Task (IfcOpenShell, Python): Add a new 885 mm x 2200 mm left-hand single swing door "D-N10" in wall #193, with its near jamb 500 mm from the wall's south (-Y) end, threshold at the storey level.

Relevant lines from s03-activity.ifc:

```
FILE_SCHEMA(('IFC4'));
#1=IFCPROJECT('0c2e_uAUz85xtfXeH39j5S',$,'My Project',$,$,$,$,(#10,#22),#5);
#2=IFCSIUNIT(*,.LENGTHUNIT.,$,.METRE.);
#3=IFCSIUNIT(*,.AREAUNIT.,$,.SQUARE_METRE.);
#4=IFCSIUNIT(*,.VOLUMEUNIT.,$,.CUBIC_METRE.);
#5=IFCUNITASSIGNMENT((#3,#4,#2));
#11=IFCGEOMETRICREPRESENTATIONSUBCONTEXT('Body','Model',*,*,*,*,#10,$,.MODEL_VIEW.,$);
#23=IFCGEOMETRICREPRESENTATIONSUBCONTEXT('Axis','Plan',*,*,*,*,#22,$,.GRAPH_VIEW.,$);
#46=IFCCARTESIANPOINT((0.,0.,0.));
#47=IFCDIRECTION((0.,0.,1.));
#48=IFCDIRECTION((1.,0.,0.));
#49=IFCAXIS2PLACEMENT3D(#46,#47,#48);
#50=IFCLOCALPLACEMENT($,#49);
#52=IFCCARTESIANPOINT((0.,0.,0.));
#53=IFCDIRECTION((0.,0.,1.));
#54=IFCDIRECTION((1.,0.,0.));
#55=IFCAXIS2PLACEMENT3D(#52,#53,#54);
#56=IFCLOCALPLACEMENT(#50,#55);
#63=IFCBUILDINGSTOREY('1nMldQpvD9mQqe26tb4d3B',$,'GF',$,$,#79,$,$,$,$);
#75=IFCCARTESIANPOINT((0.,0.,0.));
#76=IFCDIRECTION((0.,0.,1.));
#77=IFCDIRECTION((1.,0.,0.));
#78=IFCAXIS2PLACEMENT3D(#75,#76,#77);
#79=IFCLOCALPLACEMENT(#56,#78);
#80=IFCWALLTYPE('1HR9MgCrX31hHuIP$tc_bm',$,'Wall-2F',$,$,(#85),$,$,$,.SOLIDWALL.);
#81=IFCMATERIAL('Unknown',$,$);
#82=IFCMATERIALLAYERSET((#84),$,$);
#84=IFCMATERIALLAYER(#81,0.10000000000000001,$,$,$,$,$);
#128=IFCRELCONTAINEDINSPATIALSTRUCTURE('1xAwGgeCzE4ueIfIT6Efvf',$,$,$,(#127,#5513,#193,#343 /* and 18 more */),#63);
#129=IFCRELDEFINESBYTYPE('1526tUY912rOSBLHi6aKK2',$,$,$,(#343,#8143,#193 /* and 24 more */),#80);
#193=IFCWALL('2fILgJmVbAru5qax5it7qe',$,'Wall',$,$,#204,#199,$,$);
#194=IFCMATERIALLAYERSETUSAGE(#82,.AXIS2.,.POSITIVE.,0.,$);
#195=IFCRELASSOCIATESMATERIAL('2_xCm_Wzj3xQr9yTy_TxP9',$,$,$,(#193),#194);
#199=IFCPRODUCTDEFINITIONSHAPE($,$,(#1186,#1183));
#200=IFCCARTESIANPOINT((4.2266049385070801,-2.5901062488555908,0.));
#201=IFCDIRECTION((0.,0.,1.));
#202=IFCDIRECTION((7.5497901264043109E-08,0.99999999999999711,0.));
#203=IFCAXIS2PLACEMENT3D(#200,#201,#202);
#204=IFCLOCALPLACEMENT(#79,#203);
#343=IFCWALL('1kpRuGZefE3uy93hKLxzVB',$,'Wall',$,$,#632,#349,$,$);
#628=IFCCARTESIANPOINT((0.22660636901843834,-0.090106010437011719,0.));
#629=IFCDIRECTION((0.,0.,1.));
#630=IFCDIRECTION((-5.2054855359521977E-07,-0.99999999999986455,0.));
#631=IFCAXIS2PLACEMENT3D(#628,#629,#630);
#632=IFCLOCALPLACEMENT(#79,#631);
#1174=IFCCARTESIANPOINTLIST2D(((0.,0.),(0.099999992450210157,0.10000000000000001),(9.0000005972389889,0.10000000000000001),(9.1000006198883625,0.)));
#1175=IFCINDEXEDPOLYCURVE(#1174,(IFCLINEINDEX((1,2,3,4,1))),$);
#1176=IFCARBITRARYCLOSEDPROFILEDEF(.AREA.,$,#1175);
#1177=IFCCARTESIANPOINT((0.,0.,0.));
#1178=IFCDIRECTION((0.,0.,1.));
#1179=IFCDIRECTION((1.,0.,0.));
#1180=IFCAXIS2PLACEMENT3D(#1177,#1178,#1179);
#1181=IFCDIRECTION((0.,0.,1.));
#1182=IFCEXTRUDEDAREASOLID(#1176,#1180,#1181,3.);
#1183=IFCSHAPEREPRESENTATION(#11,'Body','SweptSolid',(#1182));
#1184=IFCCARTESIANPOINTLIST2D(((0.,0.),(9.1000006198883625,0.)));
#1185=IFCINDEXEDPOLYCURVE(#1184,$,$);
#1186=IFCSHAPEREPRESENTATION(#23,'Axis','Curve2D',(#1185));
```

```python
import numpy as np
import ifcopenshell
import ifcopenshell.api.feature
import ifcopenshell.api.geometry
import ifcopenshell.api.root
import ifcopenshell.api.spatial
import ifcopenshell.geom
import ifcopenshell.util.element
import ifcopenshell.util.placement
import ifcopenshell.util.representation
import ifcopenshell.util.shape
import ifcopenshell.util.unit

model = ifcopenshell.open("s03-activity.ifc")
unit_scale = ifcopenshell.util.unit.calculate_unit_scale(model)
settings = ifcopenshell.geom.settings()


def volume(element):
    """Net volume in cubic metres, openings subtracted."""
    shape = ifcopenshell.geom.create_shape(settings, element)
    return ifcopenshell.util.shape.get_volume(shape.geometry)


wall = model.by_guid("2fILgJmVbAru5qax5it7qe")
storey = ifcopenshell.util.element.get_container(wall, ifc_class="IfcBuildingStorey")
context = ifcopenshell.util.representation.get_context(model, "Model", "Body", "MODEL_VIEW")
before = volume(wall)

width, height, from_end, sill = 0.885, 2.2, 0.5, 0.0  # metres

# The wall runs along its own X axis, and the end named is its -X end.
wall_shape = ifcopenshell.geom.create_shape(settings, wall)
x, y, z = ifcopenshell.util.shape.get_vertices(wall_shape.geometry).T
start = x.min() + from_end
face, thickness = float(y.min()), float(y.max() - y.min())
wall_matrix = ifcopenshell.util.placement.get_local_placement(wall.ObjectPlacement)
level = ifcopenshell.util.placement.get_local_placement(storey.ObjectPlacement)[2, 3]


def in_wall(x, y):
    """Placement at x, y metres in the wall's axes, at sill height."""
    matrix = wall_matrix.copy()
    matrix[:, 3] = wall_matrix @ np.array([x / unit_scale, y / unit_scale, 0.0, 1.0])
    matrix[2, 3] = level + sill / unit_scale
    return matrix


# Opening: a box that overshoots both wall faces by 50 mm.
opening = ifcopenshell.api.root.create_entity(model, ifc_class="IfcOpeningElement", predefined_type="OPENING")
box = ifcopenshell.api.geometry.add_wall_representation(
    model, context=context, length=width, height=height, thickness=thickness + 0.1
)
ifcopenshell.api.geometry.assign_representation(model, product=opening, representation=box)
ifcopenshell.api.geometry.edit_object_placement(model, product=opening, matrix=in_wall(start, face - 0.05), is_si=False)
ifcopenshell.api.feature.add_feature(model, feature=opening, element=wall)

door = ifcopenshell.api.root.create_entity(model, ifc_class="IfcDoor", name="D-N10", predefined_type="DOOR")
door.OverallWidth, door.OverallHeight = width / unit_scale, height / unit_scale
door.OperationType = "SINGLE_SWING_LEFT"
body = ifcopenshell.api.geometry.add_door_representation(
    model,
    context=context,
    overall_width=door.OverallWidth,
    overall_height=door.OverallHeight,
    operation_type="SINGLE_SWING_LEFT",
    lining_properties={"LiningDepth": thickness / unit_scale, "ThresholdDepth": thickness / unit_scale},
)
ifcopenshell.api.geometry.assign_representation(model, product=door, representation=body)
ifcopenshell.api.spatial.assign_container(model, products=[door], relating_structure=storey)
ifcopenshell.api.feature.add_filling(model, opening=opening, element=door)

# The lining spans the wall, so the door starts at the wall face.
ifcopenshell.api.geometry.edit_object_placement(model, product=door, matrix=in_wall(start, face), is_si=False)

after = volume(wall)

print(f"wall volume {before:.3f} -> {after:.3f} m3")

model.write("s03-activity_updated.ifc")
```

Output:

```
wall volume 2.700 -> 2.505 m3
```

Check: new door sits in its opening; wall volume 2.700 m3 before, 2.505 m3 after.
